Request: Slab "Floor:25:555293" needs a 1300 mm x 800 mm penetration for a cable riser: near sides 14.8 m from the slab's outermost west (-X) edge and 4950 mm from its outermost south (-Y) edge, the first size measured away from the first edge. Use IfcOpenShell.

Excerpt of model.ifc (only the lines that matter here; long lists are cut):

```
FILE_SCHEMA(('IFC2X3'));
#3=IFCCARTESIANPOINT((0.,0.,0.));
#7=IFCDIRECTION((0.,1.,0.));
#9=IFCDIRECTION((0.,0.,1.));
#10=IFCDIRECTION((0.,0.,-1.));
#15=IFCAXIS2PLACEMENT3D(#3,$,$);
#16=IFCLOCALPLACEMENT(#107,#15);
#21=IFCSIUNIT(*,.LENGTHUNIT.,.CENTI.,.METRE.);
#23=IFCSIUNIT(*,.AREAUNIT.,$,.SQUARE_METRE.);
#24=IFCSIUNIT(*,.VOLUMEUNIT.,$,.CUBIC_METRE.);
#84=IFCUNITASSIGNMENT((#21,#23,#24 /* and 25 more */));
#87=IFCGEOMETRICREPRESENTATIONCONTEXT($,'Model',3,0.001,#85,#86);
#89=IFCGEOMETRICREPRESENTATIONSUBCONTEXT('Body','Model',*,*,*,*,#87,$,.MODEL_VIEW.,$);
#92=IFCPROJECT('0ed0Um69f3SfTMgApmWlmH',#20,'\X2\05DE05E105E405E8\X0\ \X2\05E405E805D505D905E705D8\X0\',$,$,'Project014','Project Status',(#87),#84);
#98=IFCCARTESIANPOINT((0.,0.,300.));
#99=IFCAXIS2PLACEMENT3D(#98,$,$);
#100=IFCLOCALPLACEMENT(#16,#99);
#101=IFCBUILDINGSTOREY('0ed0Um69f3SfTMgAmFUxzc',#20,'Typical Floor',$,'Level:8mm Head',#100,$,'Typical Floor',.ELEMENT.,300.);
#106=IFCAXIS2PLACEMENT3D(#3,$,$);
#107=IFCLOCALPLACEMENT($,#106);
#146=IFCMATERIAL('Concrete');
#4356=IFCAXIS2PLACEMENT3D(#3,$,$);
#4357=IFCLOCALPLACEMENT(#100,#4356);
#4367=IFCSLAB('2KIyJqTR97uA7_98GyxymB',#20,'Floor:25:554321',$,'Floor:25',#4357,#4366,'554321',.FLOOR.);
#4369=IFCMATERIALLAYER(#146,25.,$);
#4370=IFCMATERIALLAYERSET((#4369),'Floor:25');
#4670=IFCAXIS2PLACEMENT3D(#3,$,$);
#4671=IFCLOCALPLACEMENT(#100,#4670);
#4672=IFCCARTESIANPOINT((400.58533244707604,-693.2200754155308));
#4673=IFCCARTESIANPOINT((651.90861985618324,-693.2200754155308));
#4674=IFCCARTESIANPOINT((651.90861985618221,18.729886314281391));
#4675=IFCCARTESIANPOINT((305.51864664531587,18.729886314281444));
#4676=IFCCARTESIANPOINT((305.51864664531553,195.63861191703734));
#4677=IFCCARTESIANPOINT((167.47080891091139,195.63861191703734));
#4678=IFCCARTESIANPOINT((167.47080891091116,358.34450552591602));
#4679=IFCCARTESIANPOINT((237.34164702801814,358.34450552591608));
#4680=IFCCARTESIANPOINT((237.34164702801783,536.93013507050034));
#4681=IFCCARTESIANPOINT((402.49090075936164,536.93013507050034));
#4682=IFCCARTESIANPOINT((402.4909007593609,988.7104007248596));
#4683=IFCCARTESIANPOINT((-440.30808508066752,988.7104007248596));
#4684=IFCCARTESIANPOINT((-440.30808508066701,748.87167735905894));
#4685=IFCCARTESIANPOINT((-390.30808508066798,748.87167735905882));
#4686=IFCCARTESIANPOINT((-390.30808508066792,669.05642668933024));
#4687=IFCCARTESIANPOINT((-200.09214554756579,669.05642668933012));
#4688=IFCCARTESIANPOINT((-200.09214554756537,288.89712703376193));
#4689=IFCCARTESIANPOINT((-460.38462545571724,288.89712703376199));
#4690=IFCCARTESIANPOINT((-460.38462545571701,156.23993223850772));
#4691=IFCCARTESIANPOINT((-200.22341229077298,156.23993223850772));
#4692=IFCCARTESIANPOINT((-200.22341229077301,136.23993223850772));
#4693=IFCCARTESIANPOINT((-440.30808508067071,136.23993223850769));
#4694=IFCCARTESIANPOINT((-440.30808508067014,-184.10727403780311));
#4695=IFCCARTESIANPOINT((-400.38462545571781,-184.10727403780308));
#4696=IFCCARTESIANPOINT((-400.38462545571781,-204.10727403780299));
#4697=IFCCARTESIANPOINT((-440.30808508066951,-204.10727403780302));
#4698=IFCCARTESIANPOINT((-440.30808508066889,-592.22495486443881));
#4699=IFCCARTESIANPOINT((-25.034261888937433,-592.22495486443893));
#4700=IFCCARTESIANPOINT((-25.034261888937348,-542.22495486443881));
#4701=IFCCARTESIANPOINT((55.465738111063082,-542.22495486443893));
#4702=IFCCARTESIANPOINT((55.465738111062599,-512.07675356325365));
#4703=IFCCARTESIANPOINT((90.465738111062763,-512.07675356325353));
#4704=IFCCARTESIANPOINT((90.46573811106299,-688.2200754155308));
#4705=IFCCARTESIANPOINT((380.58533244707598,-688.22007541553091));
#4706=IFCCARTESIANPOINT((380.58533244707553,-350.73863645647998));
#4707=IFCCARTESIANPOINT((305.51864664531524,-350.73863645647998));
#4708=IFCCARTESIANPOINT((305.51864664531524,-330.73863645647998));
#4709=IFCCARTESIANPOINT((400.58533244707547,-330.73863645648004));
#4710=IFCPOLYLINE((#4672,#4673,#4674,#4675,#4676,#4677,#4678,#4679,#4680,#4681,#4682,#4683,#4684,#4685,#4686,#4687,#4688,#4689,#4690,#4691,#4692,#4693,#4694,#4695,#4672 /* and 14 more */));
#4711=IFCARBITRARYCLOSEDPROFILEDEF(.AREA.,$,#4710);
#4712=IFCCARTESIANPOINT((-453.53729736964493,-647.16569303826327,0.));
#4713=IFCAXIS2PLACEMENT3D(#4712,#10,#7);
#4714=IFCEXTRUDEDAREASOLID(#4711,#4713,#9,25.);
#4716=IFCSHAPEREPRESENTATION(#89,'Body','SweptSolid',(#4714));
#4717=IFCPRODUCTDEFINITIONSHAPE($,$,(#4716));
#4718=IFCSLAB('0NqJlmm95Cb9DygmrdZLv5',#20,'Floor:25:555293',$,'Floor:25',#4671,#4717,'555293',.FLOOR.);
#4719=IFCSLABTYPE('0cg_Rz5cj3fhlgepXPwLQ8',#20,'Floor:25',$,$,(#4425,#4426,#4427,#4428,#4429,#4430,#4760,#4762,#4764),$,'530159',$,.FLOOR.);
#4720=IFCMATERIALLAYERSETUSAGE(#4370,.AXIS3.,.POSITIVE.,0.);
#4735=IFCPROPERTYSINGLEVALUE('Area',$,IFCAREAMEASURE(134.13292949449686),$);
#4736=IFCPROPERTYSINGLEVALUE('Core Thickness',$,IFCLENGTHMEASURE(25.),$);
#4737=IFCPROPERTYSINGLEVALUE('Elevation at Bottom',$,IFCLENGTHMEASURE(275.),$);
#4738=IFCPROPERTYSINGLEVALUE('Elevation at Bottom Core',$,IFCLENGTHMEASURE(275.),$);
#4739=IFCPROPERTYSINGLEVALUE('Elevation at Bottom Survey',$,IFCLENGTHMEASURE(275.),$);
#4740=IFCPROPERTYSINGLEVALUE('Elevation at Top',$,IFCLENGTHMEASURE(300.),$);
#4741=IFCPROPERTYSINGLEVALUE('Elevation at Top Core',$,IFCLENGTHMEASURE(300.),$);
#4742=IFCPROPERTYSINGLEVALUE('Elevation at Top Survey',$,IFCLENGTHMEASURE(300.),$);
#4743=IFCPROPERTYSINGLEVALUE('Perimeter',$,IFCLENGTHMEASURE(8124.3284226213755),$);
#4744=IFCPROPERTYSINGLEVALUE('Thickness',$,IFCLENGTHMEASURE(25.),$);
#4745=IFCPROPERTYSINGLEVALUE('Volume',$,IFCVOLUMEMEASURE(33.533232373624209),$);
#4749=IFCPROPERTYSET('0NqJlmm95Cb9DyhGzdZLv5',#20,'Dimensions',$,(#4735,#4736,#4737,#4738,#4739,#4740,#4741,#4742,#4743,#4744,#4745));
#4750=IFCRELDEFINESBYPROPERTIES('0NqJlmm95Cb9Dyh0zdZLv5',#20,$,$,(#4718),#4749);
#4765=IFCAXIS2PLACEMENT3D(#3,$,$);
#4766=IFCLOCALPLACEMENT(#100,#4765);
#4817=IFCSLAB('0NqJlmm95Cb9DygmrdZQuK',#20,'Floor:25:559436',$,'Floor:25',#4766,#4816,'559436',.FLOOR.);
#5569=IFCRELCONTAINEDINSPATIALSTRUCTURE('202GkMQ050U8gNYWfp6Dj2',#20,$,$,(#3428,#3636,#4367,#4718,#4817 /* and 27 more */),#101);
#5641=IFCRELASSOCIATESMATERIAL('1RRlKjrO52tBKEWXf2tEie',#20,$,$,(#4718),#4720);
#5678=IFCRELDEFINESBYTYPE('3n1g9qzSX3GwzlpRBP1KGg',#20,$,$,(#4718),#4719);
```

```python
import numpy as np
import ifcopenshell
import ifcopenshell.api.feature
import ifcopenshell.api.geometry
import ifcopenshell.api.pset
import ifcopenshell.api.root
import ifcopenshell.geom
import ifcopenshell.util.element
import ifcopenshell.util.placement
import ifcopenshell.util.representation
import ifcopenshell.util.shape
import ifcopenshell.util.unit

model = ifcopenshell.open("model.ifc")
unit_scale = ifcopenshell.util.unit.calculate_unit_scale(model)
area_scale = ifcopenshell.util.unit.calculate_unit_scale(model, "AREAUNIT")
volume_scale = ifcopenshell.util.unit.calculate_unit_scale(model, "VOLUMEUNIT")
settings = ifcopenshell.geom.settings()


def volume(element):
    """Net volume in cubic metres, openings subtracted."""
    shape = ifcopenshell.geom.create_shape(settings, element)
    return ifcopenshell.util.shape.get_volume(shape.geometry)


slab = model.by_guid("0NqJlmm95Cb9DygmrdZLv5")
before = volume(slab)

# Extent in the slab's own axes, in metres. The edges named are its -X and -Y sides.
slab_shape = ifcopenshell.geom.create_shape(settings, slab)
vertices = ifcopenshell.util.shape.get_vertices(slab_shape.geometry)
x_min, y_min, bottom = vertices.min(axis=0)
top = vertices[:, 2].max()

opening = ifcopenshell.api.root.create_entity(model, ifc_class="IfcOpeningElement", name="Cable riser opening")
context = ifcopenshell.util.representation.get_context(model, "Model", "Body", "MODEL_VIEW")
width, depth = 1.3, 0.8
outline = [(0.0, 0.0), (width, 0.0), (width, depth), (0.0, depth), (0.0, 0.0)]
# Overshoot both faces by 50 mm so the cut is clean.
shape = ifcopenshell.api.geometry.add_slab_representation(
    model, context=context, depth=top - bottom + 0.1, polyline=outline
)
ifcopenshell.api.geometry.assign_representation(model, product=opening, representation=shape)

matrix = ifcopenshell.util.placement.get_local_placement(slab.ObjectPlacement)
matrix[:, 3] = matrix @ np.append(np.array([x_min + 14.8, y_min + 4.95, bottom - 0.05]) / unit_scale, 1.0)
ifcopenshell.api.geometry.edit_object_placement(model, product=opening, matrix=matrix, is_si=False)
ifcopenshell.api.feature.add_feature(model, feature=opening, element=slab)

after = volume(slab)

# Update the slab's stored quantities.
pset = model.by_id(ifcopenshell.util.element.get_pset(slab, "Dimensions", should_inherit=False)["id"])
ifcopenshell.api.pset.edit_pset(model, pset=pset, properties={
    "Area": model.create_entity("IfcAreaMeasure", after / (top - bottom) / area_scale),
    "Volume": model.create_entity("IfcVolumeMeasure", after / volume_scale),
})

print(f"slab volume {before:.3f} -> {after:.3f} m3")

model.write("model-out.ifc")
```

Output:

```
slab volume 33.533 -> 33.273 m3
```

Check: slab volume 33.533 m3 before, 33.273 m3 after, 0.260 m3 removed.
